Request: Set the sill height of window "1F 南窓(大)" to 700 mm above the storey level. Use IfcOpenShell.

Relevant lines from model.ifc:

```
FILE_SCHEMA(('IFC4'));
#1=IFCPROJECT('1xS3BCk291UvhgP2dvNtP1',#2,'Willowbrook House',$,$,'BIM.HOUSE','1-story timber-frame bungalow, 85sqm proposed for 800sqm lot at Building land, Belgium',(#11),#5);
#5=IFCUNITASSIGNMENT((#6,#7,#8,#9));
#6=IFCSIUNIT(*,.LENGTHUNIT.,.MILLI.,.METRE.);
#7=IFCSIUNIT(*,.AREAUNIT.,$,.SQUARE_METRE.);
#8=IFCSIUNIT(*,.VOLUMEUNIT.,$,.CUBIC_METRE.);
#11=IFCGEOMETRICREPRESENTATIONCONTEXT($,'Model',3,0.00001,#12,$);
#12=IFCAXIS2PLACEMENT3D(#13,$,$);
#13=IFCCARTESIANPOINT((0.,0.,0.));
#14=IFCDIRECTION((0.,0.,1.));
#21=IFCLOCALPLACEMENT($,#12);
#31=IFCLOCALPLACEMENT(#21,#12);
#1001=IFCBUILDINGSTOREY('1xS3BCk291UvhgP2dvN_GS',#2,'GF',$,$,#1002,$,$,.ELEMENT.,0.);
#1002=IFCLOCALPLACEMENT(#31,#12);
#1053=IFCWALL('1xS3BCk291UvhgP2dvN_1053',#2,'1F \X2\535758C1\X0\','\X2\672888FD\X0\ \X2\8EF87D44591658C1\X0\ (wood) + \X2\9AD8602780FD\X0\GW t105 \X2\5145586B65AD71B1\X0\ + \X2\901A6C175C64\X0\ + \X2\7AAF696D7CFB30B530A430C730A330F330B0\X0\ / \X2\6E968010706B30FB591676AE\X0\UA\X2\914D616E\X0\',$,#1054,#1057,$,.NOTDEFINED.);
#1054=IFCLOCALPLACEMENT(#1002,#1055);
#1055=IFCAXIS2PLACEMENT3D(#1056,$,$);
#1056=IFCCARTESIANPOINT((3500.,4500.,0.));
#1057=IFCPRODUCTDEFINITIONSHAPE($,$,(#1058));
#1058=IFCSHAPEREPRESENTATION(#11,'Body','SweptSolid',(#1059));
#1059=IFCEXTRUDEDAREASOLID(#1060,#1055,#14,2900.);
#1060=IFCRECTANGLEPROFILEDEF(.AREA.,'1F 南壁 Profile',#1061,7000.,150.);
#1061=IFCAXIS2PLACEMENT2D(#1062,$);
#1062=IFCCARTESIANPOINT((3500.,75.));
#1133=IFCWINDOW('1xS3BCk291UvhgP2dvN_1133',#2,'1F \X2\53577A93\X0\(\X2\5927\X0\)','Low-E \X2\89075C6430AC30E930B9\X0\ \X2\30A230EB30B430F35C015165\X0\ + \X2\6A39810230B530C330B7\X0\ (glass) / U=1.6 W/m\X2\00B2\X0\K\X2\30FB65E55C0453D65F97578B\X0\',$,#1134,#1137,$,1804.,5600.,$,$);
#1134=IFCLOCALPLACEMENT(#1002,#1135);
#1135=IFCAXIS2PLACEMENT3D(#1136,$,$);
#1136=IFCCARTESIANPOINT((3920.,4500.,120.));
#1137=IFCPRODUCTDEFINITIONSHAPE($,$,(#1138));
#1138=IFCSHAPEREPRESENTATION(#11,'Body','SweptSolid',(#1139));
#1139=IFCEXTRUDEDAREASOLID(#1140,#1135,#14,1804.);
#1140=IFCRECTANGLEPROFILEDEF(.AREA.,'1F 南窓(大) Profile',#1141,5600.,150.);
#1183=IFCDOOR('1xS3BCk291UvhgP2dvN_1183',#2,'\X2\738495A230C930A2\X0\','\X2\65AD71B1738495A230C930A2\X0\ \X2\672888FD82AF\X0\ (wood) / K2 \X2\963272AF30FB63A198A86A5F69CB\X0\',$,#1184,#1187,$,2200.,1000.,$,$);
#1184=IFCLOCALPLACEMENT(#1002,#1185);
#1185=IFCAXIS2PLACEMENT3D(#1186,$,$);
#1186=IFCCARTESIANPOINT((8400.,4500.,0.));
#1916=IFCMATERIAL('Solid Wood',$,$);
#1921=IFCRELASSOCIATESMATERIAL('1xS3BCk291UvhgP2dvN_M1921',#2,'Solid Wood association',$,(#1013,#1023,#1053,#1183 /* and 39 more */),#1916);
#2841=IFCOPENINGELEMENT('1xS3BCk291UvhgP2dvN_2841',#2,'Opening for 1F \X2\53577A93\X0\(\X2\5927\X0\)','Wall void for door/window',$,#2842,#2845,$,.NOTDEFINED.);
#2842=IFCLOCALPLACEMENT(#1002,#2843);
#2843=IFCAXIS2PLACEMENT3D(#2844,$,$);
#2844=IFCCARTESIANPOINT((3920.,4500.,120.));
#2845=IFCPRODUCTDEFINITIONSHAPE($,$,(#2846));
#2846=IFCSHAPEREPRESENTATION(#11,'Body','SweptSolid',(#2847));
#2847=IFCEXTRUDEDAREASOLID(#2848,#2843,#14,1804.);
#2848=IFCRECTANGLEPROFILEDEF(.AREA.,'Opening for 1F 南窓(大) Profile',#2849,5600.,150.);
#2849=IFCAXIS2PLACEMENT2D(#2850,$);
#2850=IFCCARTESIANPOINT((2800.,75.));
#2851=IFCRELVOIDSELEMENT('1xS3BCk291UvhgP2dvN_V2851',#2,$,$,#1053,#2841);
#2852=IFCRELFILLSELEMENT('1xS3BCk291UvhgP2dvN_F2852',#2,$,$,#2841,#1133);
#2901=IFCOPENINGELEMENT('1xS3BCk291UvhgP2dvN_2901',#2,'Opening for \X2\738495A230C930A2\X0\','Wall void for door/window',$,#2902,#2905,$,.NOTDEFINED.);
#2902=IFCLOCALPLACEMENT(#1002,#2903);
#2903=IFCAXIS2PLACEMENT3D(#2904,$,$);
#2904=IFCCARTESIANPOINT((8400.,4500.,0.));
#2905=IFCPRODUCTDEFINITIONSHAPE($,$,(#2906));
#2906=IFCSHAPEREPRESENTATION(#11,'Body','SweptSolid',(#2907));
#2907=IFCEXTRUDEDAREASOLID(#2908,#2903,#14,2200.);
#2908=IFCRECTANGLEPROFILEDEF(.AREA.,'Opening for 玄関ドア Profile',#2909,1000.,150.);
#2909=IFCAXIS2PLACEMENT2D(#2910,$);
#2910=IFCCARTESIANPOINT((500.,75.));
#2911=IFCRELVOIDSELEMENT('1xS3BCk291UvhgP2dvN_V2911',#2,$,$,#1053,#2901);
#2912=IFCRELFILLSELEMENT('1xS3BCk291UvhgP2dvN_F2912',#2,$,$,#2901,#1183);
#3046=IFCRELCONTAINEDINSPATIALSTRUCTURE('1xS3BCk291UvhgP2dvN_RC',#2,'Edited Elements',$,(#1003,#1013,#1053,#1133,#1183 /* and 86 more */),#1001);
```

```python
import numpy as np
import ifcopenshell
import ifcopenshell.api.geometry
import ifcopenshell.geom
import ifcopenshell.util.element
import ifcopenshell.util.placement
import ifcopenshell.util.shape
import ifcopenshell.util.unit

model = ifcopenshell.open("model.ifc")
unit_scale = ifcopenshell.util.unit.calculate_unit_scale(model)

window = model.by_id(1133)
opening = window.FillsVoids[0].RelatingOpeningElement
storey = ifcopenshell.util.element.get_container(window, ifc_class="IfcBuildingStorey")
level = ifcopenshell.util.placement.get_local_placement(storey.ObjectPlacement)[2, 3]

# The opening's origin need not be at the sill, so measure its lowest point.
shape = ifcopenshell.geom.create_shape(ifcopenshell.geom.settings(), opening)
bottom = ifcopenshell.util.shape.get_shape_bottom_elevation(shape, shape.geometry) / unit_scale
dz = level + 0.7 / unit_scale - bottom

shift = np.array([0.0, 0.0, dz])
# The window is not placed relative to its opening, so move both.
for product in (opening, window):
    matrix = ifcopenshell.util.placement.get_local_placement(product.ObjectPlacement)
    matrix[:3, 3] += shift
    ifcopenshell.api.geometry.edit_object_placement(model, product=product, matrix=matrix, is_si=False)

print(f"moved by {dz * unit_scale:+.3f} m")

model.write("model_rev.ifc")
```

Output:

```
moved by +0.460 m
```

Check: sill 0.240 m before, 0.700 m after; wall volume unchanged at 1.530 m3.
